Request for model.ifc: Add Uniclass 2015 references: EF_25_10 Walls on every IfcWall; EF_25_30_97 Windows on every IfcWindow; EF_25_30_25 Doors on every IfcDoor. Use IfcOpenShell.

First a look at what the model holds.

```python
import ifcopenshell

model = ifcopenshell.open("model.ifc")
print(model.schema)
print("classifications:", [c.Name for c in model.by_type("IfcClassification")])
for ifc_class in ("IfcDoor", "IfcRoof", "IfcStair", "IfcWall", "IfcWindow"):
    print(ifc_class, len(model.by_type(ifc_class)))
```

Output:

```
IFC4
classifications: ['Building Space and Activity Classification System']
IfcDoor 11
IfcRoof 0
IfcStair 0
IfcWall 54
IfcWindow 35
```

```python
import ifcopenshell
import ifcopenshell.api.classification

model = ifcopenshell.open("model.ifc")

system = ifcopenshell.api.classification.add_classification(model, classification="Uniclass 2015")

codes = {
    "IfcWall": ("EF_25_10", "Walls"),
    "IfcWindow": ("EF_25_30_97", "Windows"),
    "IfcDoor": ("EF_25_30_25", "Doors"),
}
for ifc_class, (code, name) in codes.items():
    products = model.by_type(ifc_class)
    ifcopenshell.api.classification.add_reference(
        model, products=products, classification=system, identification=code, name=name
    )
    print(code, len(products))

model.write("model_v2.ifc")
```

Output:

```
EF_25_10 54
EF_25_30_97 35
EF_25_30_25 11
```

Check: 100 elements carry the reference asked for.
